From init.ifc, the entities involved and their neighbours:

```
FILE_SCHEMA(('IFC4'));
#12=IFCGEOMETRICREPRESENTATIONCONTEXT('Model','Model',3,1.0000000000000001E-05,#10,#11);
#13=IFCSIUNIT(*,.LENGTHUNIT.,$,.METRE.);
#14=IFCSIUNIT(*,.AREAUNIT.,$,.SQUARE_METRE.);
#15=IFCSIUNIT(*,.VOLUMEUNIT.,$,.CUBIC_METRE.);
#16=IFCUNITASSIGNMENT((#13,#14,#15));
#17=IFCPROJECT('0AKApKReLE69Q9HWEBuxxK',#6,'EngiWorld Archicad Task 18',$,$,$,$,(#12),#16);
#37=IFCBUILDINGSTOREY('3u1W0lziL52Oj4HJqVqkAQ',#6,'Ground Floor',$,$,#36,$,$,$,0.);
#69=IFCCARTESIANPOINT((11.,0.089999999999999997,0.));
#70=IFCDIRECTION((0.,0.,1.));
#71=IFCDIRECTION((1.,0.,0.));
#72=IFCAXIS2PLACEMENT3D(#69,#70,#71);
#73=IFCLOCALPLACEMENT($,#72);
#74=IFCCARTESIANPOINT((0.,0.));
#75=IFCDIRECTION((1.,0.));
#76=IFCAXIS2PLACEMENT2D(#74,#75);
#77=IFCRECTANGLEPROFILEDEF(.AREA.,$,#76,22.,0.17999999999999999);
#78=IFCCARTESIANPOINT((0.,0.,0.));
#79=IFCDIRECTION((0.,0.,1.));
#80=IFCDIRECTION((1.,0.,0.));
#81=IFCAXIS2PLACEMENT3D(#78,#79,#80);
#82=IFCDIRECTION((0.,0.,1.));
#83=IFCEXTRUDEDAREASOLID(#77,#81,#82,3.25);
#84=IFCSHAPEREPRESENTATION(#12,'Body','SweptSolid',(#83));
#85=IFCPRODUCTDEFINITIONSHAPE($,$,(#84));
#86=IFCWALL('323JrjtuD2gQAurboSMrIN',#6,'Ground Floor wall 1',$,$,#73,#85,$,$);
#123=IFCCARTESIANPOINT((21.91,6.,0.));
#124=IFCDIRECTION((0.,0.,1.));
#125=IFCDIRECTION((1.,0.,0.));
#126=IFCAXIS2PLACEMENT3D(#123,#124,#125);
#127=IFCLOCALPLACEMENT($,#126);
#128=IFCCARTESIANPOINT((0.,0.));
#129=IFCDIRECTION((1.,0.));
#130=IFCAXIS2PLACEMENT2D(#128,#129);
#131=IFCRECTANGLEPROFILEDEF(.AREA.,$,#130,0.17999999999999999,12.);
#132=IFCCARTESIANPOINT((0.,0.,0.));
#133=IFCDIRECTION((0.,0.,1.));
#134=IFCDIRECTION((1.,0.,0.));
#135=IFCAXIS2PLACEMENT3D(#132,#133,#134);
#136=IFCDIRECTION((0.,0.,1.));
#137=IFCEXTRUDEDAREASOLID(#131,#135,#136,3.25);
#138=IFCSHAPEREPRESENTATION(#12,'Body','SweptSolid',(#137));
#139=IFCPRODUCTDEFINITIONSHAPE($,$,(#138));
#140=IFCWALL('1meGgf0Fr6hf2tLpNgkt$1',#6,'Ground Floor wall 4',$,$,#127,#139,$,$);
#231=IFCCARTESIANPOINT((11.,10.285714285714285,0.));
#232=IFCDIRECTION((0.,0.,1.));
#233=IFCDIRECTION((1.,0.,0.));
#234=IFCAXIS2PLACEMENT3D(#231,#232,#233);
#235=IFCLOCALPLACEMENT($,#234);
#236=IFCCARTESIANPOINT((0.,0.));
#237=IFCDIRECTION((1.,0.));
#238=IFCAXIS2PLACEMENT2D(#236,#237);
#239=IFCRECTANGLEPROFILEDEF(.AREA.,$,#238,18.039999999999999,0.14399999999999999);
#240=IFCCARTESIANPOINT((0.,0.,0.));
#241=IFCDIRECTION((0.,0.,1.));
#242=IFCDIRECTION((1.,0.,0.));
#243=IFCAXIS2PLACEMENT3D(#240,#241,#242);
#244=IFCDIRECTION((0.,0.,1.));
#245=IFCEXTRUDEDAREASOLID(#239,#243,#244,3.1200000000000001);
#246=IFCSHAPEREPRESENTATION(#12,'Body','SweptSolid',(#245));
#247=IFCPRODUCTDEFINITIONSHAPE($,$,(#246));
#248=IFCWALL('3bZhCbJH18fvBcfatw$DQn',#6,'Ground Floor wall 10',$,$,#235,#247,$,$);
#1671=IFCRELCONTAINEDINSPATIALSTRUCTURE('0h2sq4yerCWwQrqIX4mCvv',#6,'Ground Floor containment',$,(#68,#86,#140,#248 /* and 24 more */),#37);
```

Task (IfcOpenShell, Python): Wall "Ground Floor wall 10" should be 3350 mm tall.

```python
import ifcopenshell
import ifcopenshell.geom
import ifcopenshell.util.shape
import ifcopenshell.util.unit

model = ifcopenshell.open("init.ifc")
unit_scale = ifcopenshell.util.unit.calculate_unit_scale(model)
settings = ifcopenshell.geom.settings()


def volume(element):
    """Net volume in cubic metres, openings subtracted."""
    shape = ifcopenshell.geom.create_shape(settings, element)
    return ifcopenshell.util.shape.get_volume(shape.geometry)


wall = model.by_guid("3bZhCbJH18fvBcfatw$DQn")
before = volume(wall)

body = next(r for r in wall.Representation.Representations if r.RepresentationIdentifier == "Body")
solid = body.Items[0]
old_height = solid.Depth
solid.Depth = 3.35 / unit_scale
after = volume(wall)

print(f"height {old_height:g} -> {solid.Depth:g}, volume {before:.3f} -> {after:.3f} m3")

model.write("init_v2.ifc")
```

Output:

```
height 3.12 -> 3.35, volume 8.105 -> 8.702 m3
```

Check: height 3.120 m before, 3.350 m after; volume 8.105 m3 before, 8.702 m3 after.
